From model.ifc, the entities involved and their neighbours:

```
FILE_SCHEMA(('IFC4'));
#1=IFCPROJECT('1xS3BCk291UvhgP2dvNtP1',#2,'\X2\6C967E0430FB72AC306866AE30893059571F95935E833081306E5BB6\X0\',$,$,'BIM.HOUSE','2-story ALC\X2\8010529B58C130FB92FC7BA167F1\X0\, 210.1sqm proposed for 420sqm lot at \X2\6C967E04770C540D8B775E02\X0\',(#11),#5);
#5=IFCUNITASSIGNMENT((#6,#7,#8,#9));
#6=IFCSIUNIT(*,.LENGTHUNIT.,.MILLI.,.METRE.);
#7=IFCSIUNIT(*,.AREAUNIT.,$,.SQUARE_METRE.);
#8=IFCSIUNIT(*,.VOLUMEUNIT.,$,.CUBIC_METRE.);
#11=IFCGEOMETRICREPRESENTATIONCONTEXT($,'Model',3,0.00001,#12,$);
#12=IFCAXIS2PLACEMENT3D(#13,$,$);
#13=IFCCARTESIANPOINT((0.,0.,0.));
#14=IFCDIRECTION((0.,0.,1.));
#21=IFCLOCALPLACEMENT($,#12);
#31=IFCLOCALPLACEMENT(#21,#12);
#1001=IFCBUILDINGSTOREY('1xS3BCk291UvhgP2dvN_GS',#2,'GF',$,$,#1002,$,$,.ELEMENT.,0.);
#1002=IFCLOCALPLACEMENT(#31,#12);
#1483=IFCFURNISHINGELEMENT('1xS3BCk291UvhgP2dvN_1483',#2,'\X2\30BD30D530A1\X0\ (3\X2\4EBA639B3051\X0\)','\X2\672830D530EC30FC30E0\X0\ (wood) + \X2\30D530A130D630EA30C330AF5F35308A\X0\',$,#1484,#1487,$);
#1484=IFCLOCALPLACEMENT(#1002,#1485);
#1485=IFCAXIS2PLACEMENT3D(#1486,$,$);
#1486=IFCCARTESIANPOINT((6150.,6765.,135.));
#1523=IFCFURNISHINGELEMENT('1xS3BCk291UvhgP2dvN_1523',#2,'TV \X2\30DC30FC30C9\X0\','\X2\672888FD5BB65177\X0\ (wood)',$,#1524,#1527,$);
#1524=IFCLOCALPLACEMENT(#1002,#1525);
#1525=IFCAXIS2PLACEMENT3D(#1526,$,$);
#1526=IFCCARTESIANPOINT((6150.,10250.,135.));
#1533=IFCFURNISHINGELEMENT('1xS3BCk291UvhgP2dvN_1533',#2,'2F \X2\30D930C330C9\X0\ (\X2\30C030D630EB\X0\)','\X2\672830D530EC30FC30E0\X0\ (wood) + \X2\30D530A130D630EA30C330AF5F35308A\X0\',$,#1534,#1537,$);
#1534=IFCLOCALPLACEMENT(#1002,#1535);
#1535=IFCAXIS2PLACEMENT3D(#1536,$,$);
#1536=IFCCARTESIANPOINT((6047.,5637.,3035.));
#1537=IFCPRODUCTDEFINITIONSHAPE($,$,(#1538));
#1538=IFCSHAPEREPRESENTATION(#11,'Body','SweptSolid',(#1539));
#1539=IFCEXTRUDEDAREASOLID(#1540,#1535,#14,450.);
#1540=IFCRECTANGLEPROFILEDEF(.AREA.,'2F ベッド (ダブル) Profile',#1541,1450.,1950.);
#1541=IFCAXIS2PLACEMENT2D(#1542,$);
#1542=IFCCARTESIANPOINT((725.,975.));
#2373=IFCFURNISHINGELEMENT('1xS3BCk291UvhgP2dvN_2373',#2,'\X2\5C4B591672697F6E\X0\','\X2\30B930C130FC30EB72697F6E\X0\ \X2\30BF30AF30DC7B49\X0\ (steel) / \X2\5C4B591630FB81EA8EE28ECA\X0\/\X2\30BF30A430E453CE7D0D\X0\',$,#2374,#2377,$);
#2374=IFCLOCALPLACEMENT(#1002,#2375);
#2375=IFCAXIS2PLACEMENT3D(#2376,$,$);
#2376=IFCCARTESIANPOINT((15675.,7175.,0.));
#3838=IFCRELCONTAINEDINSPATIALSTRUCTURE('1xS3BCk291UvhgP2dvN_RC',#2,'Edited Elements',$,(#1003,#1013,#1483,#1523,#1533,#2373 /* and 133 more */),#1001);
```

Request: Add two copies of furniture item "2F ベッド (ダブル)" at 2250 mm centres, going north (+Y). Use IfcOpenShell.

```python
import numpy as np
import ifcopenshell
import ifcopenshell.api.geometry
import ifcopenshell.api.root
import ifcopenshell.util.element
import ifcopenshell.util.placement
import ifcopenshell.util.unit

model = ifcopenshell.open("model.ifc")
unit_scale = ifcopenshell.util.unit.calculate_unit_scale(model)


def reuse_history(source, copy):
    """copy_class also copies each property set's owner history, people and application; keep the originals."""
    for rel in copy.IsDefinedBy:
        if rel.is_a("IfcRelDefinesByProperties") and (history := rel.RelatingPropertyDefinition.OwnerHistory):
            rel.RelatingPropertyDefinition.OwnerHistory = source.OwnerHistory
            ifcopenshell.util.element.remove_deep2(model, history)


source = model.by_id(1533)
base = ifcopenshell.util.placement.get_local_placement(source.ObjectPlacement)
step = np.array([0.0, 1.0, 0.0]) * 2.25 / unit_scale

for i in range(1, 3):
    copy = ifcopenshell.api.root.copy_class(model, product=source)
    copy.Representation = ifcopenshell.util.element.copy_deep(
        model, source.Representation, exclude=["IfcGeometricRepresentationContext", "IfcRepresentationMap"]
    )
    reuse_history(source, copy)
    matrix = base.copy()
    matrix[:3, 3] += i * step
    print("added at", matrix[:3, 3].round(3) + 0.0)
    ifcopenshell.api.geometry.edit_object_placement(model, product=copy, matrix=matrix, is_si=False)

model.write("model_updated.ifc")
```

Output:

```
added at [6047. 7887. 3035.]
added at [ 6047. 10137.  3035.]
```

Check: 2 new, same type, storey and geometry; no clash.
